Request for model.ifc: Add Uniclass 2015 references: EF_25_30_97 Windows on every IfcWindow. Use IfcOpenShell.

First a look at what the model holds.

```python
import ifcopenshell

model = ifcopenshell.open("model.ifc")
print(model.schema)
print("classifications:", [c.Name for c in model.by_type("IfcClassification")])
for ifc_class in ("IfcDoor", "IfcRoof", "IfcStair", "IfcWall", "IfcWindow"):
    print(ifc_class, len(model.by_type(ifc_class)))
```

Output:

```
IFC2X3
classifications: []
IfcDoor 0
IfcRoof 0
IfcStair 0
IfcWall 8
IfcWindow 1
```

```python
import ifcopenshell
import ifcopenshell.api.classification

model = ifcopenshell.open("model.ifc")

# IFC2X3 requires Source and Edition and has no link from the project to the system.
system = model.create_entity("IfcClassification", Source="NBS", Edition="2015", Name="Uniclass 2015")

codes = {
    "IfcWindow": ("EF_25_30_97", "Windows"),
}
for ifc_class, (code, name) in codes.items():
    products = model.by_type(ifc_class)
    ifcopenshell.api.classification.add_reference(
        model, products=products, classification=system, identification=code, name=name
    )
    print(code, len(products))

model.write("model-out.ifc")
```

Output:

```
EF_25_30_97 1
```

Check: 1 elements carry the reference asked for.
